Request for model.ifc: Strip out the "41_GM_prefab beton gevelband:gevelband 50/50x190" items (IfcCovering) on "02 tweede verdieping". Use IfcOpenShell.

First a look at what the model holds.

```python
import ifcopenshell
import ifcopenshell.util.element

model = ifcopenshell.open("model.ifc")
print(model.schema)
storey = next(s for s in model.by_type("IfcBuildingStorey") if s.Name == "02 tweede verdieping")
coverings = [e for e in ifcopenshell.util.element.get_decomposition(storey) if e.is_a("IfcCovering")]
seen = {}
for e in coverings:
    element_type = ifcopenshell.util.element.get_type(e)
    name = element_type.Name if element_type not in (None, e) else None
    seen[name] = seen.get(name, 0) + 1
for name, count in sorted(seen.items(), key=str):
    print(count, "x", name)
```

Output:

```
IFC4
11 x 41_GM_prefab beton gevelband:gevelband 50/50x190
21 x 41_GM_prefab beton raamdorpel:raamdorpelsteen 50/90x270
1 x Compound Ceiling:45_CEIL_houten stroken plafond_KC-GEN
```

```python
import ifcopenshell
import ifcopenshell.api.root
import ifcopenshell.util.element

model = ifcopenshell.open("model.ifc")

storey = next(s for s in model.by_type("IfcBuildingStorey") if s.Name == "02 tweede verdieping")
coverings = [e for e in ifcopenshell.util.element.get_decomposition(storey) if e.is_a("IfcCovering")]
targets = [e for e in coverings if (t := ifcopenshell.util.element.get_type(e)) not in (None, e) and t.Name == "41_GM_prefab beton gevelband:gevelband 50/50x190"]

for e in targets:
    ifcopenshell.api.root.remove_product(model, product=e)
print(len(targets), "removed")

model.write("model_v2.ifc")
```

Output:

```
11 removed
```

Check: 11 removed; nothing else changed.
